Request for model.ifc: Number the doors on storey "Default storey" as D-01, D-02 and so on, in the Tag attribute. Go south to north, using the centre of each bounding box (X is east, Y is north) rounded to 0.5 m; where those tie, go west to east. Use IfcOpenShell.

First a look at what the model holds.

```python
import ifcopenshell
import ifcopenshell.util.element
import ifcopenshell.util.placement

model = ifcopenshell.open("model.ifc")
print(model.schema)
storey = next(s for s in model.by_type("IfcBuildingStorey") if s.Name == "Default storey")
doors = [e for e in ifcopenshell.util.element.get_decomposition(storey) if e.is_a("IfcDoor")]
for e in sorted(doors, key=lambda e: e.id()):
    origin = ifcopenshell.util.placement.get_local_placement(e.ObjectPlacement)[:3, 3]
    print(e.id(), e.Tag, e.Name, origin.round(2) + 0.0, sep=" | ")
```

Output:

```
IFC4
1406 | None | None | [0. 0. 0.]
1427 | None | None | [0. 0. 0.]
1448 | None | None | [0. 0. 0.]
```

```python
import ifcopenshell
import ifcopenshell.geom
import ifcopenshell.util.element
import ifcopenshell.util.shape

model = ifcopenshell.open("model.ifc")
settings = ifcopenshell.geom.settings()
settings.set("use-world-coords", True)


def centre(element):
    shape = ifcopenshell.geom.create_shape(settings, element)
    return ifcopenshell.util.shape.get_bbox_centroid(shape.geometry)


storey = next(s for s in model.by_type("IfcBuildingStorey") if s.Name == "Default storey")
doors = [e for e in ifcopenshell.util.element.get_decomposition(storey) if e.is_a("IfcDoor")]

# Insertion points can sit at a corner or the storey origin, so sort by the geometry (in metres).
centres = {e: centre(e) for e in doors}
doors.sort(key=lambda e: (round(centres[e][1] / 0.5), centres[e][0]))

for i, e in enumerate(doors, start=1):
    number = f"D-{i:02d}"
    e.Tag = number
    print(e.id(), number)

model.write("model-out.ifc")
```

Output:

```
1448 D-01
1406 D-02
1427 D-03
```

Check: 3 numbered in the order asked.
